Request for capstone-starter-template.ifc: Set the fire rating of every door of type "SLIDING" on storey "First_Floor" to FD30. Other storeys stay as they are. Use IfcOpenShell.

First a look at what the model holds.

```python
import ifcopenshell
import ifcopenshell.util.element

model = ifcopenshell.open("capstone-starter-template.ifc")
print(model.schema)
storey = next(s for s in model.by_type("IfcBuildingStorey") if s.Name == "First_Floor")
doors = [e for e in ifcopenshell.util.element.get_decomposition(storey) if e.is_a("IfcDoor")]
seen = {}
for e in doors:
    element_type = ifcopenshell.util.element.get_type(e)
    key = (element_type.Name if element_type != e and element_type else None, ifcopenshell.util.element.get_pset(e, "Pset_DoorCommon", "FireRating"))
    seen[key] = seen.get(key, 0) + 1
for (name, value), count in sorted(seen.items(), key=str):
    print(count, "x", name, "|", value)
```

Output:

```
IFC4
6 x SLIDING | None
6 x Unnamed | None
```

```python
import ifcopenshell
import ifcopenshell.api.pset
import ifcopenshell.util.element

model = ifcopenshell.open("capstone-starter-template.ifc")

storey = next(s for s in model.by_type("IfcBuildingStorey") if s.Name == "First_Floor")
doors = [e for e in ifcopenshell.util.element.get_decomposition(storey) if e.is_a("IfcDoor")]

count = 0
for e in doors:
    element_type = ifcopenshell.util.element.get_type(e)
    if element_type in (None, e) or element_type.Name != "SLIDING":
        continue
    # add_pset returns the element's existing set when there is one.
    pset = ifcopenshell.api.pset.add_pset(model, product=e, name="Pset_DoorCommon")
    ifcopenshell.api.pset.edit_pset(model, pset=pset, properties={"FireRating": "FD30"})
    count += 1

print(count, "doors updated")

model.write("capstone-starter-template_v2.ifc")
```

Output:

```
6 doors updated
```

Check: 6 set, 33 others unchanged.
